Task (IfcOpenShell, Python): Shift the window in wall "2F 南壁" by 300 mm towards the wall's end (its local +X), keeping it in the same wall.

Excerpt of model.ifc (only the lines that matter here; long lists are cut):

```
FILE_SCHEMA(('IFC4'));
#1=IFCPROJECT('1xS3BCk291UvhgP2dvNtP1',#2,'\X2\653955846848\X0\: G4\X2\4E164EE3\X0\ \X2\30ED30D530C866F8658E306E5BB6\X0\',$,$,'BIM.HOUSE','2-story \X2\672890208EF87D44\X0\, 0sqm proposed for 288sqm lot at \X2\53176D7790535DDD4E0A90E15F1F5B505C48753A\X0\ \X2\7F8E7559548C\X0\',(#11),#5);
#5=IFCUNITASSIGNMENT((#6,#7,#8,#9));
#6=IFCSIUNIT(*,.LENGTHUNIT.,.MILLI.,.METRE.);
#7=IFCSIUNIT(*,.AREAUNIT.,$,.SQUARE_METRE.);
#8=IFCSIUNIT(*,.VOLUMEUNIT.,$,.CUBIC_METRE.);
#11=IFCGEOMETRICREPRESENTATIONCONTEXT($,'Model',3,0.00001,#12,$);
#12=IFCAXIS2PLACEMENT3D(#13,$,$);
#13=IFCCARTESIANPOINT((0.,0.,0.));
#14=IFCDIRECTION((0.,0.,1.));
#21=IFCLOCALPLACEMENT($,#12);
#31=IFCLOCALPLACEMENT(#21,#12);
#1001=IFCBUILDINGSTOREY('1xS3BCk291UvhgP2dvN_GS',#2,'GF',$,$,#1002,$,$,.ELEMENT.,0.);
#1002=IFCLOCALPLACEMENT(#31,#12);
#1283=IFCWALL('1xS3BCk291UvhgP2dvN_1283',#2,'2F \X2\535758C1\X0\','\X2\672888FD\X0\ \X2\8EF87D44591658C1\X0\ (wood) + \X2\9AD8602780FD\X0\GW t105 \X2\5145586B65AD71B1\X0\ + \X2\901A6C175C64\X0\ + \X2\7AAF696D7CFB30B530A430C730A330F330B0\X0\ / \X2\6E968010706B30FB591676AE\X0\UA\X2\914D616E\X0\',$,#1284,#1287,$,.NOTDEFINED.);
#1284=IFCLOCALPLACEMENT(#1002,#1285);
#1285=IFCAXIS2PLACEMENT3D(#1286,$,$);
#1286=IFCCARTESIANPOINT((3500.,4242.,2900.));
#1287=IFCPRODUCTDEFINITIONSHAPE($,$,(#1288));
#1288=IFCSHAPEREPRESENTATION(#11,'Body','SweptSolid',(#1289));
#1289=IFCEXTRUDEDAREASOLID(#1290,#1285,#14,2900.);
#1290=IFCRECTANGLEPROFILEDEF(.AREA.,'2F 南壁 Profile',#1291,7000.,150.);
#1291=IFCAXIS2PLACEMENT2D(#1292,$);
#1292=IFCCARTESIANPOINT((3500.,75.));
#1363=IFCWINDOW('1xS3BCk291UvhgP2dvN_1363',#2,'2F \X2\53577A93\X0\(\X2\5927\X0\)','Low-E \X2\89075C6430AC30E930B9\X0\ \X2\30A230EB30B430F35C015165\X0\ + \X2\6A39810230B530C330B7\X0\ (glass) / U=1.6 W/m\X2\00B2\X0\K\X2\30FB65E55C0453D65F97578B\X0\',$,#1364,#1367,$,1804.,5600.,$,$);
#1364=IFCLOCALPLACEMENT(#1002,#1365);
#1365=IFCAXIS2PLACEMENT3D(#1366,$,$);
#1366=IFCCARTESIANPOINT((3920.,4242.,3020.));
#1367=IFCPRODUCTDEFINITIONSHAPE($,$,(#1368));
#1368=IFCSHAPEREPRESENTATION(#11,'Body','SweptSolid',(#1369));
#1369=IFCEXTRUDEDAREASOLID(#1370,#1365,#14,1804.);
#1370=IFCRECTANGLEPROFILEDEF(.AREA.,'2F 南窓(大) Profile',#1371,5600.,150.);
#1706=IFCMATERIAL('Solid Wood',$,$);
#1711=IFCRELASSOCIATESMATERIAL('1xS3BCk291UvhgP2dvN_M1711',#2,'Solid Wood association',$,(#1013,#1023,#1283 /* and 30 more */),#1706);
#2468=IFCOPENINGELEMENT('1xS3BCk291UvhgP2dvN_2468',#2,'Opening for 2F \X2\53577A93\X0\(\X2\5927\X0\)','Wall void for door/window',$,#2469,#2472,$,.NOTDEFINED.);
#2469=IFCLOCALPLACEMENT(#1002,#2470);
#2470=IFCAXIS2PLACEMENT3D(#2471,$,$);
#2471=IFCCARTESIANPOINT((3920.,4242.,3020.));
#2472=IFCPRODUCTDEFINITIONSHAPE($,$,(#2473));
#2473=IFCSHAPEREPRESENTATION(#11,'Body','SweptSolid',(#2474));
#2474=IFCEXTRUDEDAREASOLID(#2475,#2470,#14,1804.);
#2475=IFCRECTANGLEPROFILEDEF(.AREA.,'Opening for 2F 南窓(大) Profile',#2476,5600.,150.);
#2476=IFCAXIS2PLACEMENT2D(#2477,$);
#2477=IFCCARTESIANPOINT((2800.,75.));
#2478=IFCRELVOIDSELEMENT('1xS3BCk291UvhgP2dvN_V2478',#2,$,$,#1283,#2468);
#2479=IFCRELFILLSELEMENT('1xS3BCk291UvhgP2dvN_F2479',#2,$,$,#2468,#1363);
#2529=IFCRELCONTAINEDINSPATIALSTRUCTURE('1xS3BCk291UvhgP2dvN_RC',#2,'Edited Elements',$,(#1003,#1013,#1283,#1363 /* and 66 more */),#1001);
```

```python
import ifcopenshell
import ifcopenshell.api.geometry
import ifcopenshell.util.placement

model = ifcopenshell.open("model.ifc")

window = model.by_guid("1xS3BCk291UvhgP2dvN_1363")
opening = window.FillsVoids[0].RelatingOpeningElement
wall = opening.VoidsElements[0].RelatingBuildingElement

wall_matrix = ifcopenshell.util.placement.get_local_placement(wall.ObjectPlacement)
shift = wall_matrix[:3, 0] * 300.0
before = ifcopenshell.util.placement.get_local_placement(window.ObjectPlacement)[:3, 3].copy()

# The window is not placed relative to its opening, so move both.
for product in (opening, window):
    matrix = ifcopenshell.util.placement.get_local_placement(product.ObjectPlacement)
    matrix[:3, 3] += shift
    ifcopenshell.api.geometry.edit_object_placement(model, product=product, matrix=matrix, is_si=False)

after = ifcopenshell.util.placement.get_local_placement(window.ObjectPlacement)[:3, 3]
print("window moved by", (after - before).round(3) + 0.0)

model.write("model_updated.ifc")
```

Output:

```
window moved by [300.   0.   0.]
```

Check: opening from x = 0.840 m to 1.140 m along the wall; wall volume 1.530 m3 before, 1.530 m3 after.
